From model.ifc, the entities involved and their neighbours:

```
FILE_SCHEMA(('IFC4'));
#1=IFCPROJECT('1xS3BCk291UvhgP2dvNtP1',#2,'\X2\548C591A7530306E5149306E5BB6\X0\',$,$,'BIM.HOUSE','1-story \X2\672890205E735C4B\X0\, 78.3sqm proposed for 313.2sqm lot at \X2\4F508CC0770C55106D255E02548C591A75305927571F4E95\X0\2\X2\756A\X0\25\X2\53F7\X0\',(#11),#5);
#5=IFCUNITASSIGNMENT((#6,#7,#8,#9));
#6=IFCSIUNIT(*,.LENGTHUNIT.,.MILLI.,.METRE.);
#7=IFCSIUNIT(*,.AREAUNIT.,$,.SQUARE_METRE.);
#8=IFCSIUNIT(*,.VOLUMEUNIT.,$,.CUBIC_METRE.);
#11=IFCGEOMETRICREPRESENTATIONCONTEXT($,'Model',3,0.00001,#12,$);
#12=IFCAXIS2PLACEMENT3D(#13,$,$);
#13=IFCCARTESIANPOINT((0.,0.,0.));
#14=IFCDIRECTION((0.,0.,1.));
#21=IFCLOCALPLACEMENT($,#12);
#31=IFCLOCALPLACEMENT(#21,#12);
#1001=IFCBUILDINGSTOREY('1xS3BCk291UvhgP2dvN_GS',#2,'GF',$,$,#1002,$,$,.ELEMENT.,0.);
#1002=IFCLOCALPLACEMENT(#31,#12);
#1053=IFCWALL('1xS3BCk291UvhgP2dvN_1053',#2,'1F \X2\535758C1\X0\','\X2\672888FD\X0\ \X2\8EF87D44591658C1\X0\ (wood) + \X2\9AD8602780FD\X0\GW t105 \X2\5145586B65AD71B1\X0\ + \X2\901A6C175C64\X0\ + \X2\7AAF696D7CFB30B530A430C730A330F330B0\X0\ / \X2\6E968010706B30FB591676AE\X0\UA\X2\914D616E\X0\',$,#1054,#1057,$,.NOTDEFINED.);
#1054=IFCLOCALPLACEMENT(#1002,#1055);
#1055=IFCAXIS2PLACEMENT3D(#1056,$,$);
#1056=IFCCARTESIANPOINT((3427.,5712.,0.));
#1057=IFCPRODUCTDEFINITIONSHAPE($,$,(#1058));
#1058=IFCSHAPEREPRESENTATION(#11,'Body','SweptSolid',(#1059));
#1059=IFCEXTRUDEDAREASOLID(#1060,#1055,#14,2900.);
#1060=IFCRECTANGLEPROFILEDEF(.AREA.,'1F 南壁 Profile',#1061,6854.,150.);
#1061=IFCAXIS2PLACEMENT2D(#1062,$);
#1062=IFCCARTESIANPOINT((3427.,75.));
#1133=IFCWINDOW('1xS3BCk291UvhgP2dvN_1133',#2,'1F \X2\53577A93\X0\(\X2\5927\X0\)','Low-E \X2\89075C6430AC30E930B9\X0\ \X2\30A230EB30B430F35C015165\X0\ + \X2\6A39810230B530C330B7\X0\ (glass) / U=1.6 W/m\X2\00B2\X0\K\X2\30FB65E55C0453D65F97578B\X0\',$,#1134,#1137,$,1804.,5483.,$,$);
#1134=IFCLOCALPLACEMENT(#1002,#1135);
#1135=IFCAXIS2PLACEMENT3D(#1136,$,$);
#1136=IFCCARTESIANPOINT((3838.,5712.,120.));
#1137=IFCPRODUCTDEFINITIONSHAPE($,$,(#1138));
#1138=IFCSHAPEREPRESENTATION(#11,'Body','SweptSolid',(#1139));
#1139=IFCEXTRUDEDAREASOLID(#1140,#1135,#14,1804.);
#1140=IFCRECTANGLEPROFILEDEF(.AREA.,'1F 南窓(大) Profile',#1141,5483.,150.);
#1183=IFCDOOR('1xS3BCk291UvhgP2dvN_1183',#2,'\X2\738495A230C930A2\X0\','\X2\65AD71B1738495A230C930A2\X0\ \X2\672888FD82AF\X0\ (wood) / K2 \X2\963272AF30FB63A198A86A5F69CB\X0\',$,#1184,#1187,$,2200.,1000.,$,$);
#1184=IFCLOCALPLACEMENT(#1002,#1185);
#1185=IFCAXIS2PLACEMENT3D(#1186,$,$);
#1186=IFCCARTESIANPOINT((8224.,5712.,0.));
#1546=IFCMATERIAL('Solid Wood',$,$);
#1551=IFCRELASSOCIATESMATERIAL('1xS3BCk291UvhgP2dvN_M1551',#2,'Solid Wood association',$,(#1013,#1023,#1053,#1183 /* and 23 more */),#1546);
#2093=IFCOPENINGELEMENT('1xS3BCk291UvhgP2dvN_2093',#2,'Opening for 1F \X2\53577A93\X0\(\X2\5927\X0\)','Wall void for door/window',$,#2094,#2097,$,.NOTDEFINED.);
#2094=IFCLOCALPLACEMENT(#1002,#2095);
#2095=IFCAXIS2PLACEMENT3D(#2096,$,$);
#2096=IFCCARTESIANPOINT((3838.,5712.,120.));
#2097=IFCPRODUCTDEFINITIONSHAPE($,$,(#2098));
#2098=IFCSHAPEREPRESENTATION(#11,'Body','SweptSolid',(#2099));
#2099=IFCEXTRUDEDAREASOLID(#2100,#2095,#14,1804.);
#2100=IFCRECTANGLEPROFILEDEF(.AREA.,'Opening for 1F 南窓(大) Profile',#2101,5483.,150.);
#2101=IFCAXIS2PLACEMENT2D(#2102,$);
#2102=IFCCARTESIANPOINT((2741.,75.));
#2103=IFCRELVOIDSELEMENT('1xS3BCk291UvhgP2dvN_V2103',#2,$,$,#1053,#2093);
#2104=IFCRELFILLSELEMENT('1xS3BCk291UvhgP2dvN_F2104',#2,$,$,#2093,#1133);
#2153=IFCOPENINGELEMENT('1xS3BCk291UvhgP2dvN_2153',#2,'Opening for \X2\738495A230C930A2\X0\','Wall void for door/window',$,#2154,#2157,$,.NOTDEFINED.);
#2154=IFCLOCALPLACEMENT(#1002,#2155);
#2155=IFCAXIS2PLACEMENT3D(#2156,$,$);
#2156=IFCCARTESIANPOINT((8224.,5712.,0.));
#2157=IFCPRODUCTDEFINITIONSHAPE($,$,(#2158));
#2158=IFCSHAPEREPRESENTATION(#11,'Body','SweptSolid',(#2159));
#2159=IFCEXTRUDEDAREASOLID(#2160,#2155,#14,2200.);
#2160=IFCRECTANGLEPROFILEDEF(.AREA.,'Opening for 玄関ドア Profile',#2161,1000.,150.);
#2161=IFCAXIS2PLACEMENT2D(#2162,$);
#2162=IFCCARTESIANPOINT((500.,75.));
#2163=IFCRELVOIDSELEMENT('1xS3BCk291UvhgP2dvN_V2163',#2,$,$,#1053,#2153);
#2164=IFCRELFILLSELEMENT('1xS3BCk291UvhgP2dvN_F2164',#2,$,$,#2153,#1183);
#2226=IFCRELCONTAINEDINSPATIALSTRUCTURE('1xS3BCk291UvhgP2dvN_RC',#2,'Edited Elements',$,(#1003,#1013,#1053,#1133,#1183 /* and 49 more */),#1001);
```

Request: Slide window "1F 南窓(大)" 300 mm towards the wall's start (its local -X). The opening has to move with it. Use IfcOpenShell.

```python
import ifcopenshell
import ifcopenshell.api.geometry
import ifcopenshell.util.placement
import ifcopenshell.util.unit

model = ifcopenshell.open("model.ifc")
unit_scale = ifcopenshell.util.unit.calculate_unit_scale(model)

window = model.by_guid("1xS3BCk291UvhgP2dvN_1133")
opening = window.FillsVoids[0].RelatingOpeningElement
wall = opening.VoidsElements[0].RelatingBuildingElement

wall_matrix = ifcopenshell.util.placement.get_local_placement(wall.ObjectPlacement)
shift = wall_matrix[:3, 0] * -0.3 / unit_scale
before = ifcopenshell.util.placement.get_local_placement(window.ObjectPlacement)[:3, 3].copy()

# The window is not placed relative to its opening, so move both.
for product in (opening, window):
    matrix = ifcopenshell.util.placement.get_local_placement(product.ObjectPlacement)
    matrix[:3, 3] += shift
    ifcopenshell.api.geometry.edit_object_placement(model, product=product, matrix=matrix, is_si=False)

after = ifcopenshell.util.placement.get_local_placement(window.ObjectPlacement)[:3, 3]
print("window moved by", (after - before).round(3) + 0.0)

model.write("model_rev.ifc")
```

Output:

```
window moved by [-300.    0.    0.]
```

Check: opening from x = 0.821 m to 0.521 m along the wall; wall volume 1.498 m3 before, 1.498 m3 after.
